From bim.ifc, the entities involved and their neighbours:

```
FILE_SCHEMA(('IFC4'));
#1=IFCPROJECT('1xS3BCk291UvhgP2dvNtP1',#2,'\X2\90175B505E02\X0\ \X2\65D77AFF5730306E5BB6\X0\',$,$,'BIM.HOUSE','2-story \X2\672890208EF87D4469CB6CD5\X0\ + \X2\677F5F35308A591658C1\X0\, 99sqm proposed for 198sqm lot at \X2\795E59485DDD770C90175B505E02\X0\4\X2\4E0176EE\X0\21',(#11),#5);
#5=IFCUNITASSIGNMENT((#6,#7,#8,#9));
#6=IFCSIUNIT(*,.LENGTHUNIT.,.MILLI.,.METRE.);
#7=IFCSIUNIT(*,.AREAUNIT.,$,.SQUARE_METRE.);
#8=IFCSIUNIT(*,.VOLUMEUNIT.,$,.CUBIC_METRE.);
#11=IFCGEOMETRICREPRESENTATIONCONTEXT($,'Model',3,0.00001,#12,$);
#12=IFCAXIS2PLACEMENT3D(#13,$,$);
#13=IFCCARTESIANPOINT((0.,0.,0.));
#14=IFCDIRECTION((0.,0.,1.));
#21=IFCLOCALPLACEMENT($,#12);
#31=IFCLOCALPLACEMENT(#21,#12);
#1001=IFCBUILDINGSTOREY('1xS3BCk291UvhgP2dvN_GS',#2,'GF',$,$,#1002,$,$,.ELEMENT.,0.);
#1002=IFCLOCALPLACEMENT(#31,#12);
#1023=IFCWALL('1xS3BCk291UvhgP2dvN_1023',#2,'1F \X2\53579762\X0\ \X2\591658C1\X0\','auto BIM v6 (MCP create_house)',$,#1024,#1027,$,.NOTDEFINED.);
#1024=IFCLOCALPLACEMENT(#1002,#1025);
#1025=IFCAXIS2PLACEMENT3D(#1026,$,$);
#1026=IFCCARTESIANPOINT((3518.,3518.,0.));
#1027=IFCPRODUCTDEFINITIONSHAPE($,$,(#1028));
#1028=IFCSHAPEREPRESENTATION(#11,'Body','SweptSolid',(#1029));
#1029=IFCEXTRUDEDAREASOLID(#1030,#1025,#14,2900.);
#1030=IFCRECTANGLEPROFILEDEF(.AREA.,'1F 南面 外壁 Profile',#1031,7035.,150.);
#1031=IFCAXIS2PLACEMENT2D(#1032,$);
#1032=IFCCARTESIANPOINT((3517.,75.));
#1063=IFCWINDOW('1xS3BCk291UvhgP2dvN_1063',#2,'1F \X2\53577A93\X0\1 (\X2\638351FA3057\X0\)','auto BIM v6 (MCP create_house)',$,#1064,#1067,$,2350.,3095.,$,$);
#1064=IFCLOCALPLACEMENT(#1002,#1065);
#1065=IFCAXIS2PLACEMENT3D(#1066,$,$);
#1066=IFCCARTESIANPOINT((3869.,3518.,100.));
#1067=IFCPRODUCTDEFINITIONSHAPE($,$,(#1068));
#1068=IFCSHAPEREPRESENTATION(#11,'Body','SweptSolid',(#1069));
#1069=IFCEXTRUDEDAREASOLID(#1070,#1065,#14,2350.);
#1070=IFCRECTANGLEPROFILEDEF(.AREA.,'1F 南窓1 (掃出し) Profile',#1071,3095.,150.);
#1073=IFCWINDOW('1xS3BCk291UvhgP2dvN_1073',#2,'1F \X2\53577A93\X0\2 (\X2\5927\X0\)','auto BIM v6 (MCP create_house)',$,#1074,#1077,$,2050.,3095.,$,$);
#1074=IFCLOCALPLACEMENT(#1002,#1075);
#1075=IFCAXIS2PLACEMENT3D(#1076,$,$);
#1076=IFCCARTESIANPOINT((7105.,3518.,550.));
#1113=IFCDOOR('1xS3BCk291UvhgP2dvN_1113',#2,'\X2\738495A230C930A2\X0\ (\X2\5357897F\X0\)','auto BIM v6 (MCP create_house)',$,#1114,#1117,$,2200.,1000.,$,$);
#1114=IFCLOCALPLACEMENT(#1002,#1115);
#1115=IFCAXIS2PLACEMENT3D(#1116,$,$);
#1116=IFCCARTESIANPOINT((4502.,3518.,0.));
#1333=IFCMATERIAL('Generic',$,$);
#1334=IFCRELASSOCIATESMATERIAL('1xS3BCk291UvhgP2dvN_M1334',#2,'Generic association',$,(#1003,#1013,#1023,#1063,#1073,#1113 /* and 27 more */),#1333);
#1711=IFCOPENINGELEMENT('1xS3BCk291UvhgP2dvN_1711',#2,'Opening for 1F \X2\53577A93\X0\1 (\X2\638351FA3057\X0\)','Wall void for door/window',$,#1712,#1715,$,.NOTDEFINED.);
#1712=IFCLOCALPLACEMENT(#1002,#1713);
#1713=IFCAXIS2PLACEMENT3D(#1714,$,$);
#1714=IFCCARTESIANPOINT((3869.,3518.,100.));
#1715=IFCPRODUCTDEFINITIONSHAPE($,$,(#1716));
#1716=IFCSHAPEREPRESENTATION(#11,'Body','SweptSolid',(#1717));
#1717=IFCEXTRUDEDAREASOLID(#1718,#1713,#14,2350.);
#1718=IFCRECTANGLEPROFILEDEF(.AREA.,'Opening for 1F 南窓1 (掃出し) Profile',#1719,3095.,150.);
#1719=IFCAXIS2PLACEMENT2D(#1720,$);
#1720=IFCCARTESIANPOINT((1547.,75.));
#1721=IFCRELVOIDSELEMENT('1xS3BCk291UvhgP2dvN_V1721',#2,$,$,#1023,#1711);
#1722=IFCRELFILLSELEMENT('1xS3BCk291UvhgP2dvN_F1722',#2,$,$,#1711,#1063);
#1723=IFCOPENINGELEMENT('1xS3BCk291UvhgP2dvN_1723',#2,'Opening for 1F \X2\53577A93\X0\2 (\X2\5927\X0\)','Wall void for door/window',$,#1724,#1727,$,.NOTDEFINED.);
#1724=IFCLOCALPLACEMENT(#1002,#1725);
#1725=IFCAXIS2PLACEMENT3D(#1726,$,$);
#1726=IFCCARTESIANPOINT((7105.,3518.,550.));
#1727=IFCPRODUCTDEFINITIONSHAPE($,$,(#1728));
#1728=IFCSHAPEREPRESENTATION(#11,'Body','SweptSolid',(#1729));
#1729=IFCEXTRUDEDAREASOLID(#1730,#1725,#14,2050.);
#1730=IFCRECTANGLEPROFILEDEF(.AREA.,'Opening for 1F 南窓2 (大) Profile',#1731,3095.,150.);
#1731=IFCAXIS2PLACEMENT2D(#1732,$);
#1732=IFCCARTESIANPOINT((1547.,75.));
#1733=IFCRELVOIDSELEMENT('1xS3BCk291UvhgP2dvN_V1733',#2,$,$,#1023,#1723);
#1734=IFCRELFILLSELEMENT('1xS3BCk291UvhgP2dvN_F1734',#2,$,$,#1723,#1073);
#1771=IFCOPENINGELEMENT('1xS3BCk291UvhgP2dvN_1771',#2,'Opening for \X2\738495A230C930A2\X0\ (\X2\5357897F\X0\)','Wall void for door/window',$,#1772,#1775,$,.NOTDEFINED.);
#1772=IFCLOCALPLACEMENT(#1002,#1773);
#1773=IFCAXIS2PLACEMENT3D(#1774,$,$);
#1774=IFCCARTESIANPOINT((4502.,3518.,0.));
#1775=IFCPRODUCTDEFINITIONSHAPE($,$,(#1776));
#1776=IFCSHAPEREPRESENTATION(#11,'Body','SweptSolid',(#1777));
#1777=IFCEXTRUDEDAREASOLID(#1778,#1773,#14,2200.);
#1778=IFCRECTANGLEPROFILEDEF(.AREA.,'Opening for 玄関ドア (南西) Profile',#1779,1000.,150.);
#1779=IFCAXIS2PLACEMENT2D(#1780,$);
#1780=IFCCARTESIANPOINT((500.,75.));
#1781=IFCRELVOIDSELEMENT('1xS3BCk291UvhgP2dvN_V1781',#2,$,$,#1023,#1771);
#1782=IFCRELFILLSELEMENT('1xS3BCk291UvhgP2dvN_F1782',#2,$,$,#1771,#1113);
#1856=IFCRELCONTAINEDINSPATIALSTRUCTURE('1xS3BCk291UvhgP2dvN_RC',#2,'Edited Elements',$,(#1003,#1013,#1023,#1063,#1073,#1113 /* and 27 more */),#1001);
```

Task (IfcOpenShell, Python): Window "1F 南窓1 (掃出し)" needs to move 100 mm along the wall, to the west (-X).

```python
import ifcopenshell
import ifcopenshell.api.geometry
import ifcopenshell.util.placement
import ifcopenshell.util.unit

model = ifcopenshell.open("bim.ifc")
unit_scale = ifcopenshell.util.unit.calculate_unit_scale(model)

window = model.by_id(1063)
opening = window.FillsVoids[0].RelatingOpeningElement
wall = opening.VoidsElements[0].RelatingBuildingElement

wall_matrix = ifcopenshell.util.placement.get_local_placement(wall.ObjectPlacement)
shift = wall_matrix[:3, 0] * -0.1 / unit_scale
before = ifcopenshell.util.placement.get_local_placement(window.ObjectPlacement)[:3, 3].copy()

# The window is not placed relative to its opening, so move both.
for product in (opening, window):
    matrix = ifcopenshell.util.placement.get_local_placement(product.ObjectPlacement)
    matrix[:3, 3] += shift
    ifcopenshell.api.geometry.edit_object_placement(model, product=product, matrix=matrix, is_si=False)

after = ifcopenshell.util.placement.get_local_placement(window.ObjectPlacement)[:3, 3]
print("window moved by", (after - before).round(3) + 0.0)

model.write("bim_rev.ifc")
```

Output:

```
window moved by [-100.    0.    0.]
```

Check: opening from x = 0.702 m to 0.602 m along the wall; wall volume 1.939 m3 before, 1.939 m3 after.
